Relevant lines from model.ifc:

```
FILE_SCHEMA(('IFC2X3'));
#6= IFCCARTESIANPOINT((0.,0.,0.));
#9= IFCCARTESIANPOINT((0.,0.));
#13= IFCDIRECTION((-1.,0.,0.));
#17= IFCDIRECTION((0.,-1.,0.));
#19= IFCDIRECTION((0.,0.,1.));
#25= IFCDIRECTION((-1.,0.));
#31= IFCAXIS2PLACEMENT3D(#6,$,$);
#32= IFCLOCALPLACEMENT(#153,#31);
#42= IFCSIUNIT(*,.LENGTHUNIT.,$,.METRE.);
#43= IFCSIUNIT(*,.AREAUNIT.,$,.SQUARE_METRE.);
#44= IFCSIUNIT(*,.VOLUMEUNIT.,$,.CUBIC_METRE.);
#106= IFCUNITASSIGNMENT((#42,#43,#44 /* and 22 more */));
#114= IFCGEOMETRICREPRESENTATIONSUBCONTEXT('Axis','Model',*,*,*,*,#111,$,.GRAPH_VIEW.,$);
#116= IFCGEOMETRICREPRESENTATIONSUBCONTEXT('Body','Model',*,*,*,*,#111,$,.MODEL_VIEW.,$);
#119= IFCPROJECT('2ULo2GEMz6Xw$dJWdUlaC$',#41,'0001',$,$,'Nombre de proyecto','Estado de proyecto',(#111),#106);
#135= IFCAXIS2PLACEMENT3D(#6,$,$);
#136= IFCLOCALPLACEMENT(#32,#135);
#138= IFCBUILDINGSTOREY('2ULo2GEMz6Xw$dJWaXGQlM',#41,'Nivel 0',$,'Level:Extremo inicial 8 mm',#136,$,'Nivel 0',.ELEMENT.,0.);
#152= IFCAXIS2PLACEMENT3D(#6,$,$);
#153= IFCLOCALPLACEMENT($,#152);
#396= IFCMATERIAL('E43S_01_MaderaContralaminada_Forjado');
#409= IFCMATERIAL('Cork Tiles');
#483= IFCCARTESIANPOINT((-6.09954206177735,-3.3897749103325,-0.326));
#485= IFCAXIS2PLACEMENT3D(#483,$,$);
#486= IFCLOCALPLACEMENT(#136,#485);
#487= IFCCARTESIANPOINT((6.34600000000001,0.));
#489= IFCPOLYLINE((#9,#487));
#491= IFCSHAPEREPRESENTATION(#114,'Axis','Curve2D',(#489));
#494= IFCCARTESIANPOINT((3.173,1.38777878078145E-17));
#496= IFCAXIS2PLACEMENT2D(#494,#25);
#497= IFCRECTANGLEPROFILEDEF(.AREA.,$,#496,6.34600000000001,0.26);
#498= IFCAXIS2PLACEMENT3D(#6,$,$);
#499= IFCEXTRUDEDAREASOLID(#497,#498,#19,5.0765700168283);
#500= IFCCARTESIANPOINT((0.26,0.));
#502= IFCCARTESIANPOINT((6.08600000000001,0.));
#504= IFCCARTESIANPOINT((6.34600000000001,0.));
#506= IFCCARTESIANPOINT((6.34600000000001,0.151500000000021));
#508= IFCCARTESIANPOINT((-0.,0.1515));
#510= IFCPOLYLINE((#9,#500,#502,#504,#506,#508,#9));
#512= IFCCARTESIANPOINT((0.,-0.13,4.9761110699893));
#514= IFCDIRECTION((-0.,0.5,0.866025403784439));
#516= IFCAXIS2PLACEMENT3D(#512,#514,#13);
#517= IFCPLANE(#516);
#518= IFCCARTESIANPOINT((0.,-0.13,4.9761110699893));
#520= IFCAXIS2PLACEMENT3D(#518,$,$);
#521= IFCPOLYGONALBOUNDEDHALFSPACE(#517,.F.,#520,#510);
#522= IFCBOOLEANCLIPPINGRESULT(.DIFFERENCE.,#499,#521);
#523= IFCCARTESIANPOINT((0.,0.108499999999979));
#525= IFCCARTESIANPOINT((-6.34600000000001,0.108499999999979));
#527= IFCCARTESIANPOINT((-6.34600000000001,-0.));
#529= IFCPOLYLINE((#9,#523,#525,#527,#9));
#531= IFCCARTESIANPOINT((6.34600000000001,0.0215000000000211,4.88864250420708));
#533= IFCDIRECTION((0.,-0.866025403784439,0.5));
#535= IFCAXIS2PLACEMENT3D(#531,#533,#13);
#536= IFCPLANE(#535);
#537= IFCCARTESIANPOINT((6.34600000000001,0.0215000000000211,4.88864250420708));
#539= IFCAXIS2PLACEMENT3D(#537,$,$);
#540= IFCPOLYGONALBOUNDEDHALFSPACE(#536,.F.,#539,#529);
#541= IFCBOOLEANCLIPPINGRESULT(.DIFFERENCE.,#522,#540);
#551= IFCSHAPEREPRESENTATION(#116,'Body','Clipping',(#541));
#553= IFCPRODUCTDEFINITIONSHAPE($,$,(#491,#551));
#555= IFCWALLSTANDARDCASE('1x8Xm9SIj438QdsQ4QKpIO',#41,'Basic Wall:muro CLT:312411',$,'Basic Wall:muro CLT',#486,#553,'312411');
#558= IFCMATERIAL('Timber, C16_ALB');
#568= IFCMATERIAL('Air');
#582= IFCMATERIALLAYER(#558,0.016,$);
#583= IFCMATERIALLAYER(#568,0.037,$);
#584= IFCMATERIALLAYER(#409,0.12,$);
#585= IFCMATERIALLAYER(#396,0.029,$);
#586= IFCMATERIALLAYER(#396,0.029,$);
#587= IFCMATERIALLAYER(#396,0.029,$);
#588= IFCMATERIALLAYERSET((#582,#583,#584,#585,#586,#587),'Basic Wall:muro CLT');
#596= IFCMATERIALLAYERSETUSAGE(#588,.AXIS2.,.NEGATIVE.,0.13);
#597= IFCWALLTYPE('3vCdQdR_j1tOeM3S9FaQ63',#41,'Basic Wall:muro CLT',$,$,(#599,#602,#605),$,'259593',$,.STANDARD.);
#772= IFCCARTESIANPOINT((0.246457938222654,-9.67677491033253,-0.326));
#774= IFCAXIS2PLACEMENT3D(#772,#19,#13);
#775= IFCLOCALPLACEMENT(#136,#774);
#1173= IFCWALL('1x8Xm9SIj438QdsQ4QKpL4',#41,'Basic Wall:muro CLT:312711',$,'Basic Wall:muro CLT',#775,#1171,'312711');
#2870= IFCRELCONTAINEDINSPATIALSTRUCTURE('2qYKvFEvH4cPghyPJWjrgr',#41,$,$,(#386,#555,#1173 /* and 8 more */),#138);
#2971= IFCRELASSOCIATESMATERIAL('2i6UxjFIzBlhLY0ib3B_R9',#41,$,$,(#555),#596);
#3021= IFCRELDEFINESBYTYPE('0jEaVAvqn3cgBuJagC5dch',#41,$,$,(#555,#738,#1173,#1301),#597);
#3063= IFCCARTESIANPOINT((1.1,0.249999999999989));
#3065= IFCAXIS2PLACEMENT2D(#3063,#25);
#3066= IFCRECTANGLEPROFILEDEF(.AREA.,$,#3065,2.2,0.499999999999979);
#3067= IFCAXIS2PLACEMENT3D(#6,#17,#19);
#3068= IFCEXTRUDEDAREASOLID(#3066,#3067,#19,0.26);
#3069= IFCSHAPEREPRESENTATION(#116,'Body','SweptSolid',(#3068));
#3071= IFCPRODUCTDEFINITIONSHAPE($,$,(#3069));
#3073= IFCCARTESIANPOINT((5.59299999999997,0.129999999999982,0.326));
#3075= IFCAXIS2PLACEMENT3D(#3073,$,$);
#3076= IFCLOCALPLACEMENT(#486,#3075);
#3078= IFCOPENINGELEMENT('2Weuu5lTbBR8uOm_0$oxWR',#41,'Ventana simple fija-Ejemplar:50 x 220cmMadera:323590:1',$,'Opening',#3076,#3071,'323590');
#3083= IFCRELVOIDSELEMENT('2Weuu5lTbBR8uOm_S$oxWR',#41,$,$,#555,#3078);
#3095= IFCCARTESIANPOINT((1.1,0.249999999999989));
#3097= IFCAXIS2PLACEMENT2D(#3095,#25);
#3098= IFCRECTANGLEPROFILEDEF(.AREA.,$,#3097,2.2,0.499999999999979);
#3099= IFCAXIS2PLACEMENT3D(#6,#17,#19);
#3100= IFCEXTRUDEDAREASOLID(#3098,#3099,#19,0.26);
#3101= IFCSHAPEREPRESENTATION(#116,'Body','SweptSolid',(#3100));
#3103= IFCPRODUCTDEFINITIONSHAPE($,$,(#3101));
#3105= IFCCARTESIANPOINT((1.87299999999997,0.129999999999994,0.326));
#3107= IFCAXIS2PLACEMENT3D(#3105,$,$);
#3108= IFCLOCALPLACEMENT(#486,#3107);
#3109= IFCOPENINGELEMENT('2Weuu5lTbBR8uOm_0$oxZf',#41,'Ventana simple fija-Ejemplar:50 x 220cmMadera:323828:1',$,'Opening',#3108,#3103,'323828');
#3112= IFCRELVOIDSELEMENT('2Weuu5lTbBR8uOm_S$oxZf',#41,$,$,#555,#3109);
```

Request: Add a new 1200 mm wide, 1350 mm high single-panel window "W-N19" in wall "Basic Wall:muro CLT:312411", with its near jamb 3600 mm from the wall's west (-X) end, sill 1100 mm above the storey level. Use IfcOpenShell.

```python
import numpy as np
import ifcopenshell
import ifcopenshell.api.feature
import ifcopenshell.api.geometry
import ifcopenshell.api.root
import ifcopenshell.api.spatial
import ifcopenshell.api.type
import ifcopenshell.geom
import ifcopenshell.util.element
import ifcopenshell.util.placement
import ifcopenshell.util.representation
import ifcopenshell.util.shape
import ifcopenshell.util.unit

model = ifcopenshell.open("model.ifc")
unit_scale = ifcopenshell.util.unit.calculate_unit_scale(model)
settings = ifcopenshell.geom.settings()


def volume(element):
    """Net volume in cubic metres, openings subtracted."""
    shape = ifcopenshell.geom.create_shape(settings, element)
    return ifcopenshell.util.shape.get_volume(shape.geometry)


wall = model.by_guid("1x8Xm9SIj438QdsQ4QKpIO")
storey = ifcopenshell.util.element.get_container(wall, ifc_class="IfcBuildingStorey")
context = ifcopenshell.util.representation.get_context(model, "Model", "Body", "MODEL_VIEW")
before = volume(wall)

width, height, from_end, sill = 1.2, 1.35, 3.6, 1.1  # metres

# The wall runs along its own X axis, and the end named is its -X end.
wall_shape = ifcopenshell.geom.create_shape(settings, wall)
x, y, z = ifcopenshell.util.shape.get_vertices(wall_shape.geometry).T
start = x.min() + from_end
face, thickness = float(y.min()), float(y.max() - y.min())
wall_matrix = ifcopenshell.util.placement.get_local_placement(wall.ObjectPlacement)
level = ifcopenshell.util.placement.get_local_placement(storey.ObjectPlacement)[2, 3]


def in_wall(x, y):
    """Placement at x, y metres in the wall's axes, at sill height."""
    matrix = wall_matrix.copy()
    matrix[:, 3] = wall_matrix @ np.array([x / unit_scale, y / unit_scale, 0.0, 1.0])
    matrix[2, 3] = level + sill / unit_scale
    return matrix


# Opening: a box that overshoots both wall faces by 50 mm.
opening = ifcopenshell.api.root.create_entity(model, ifc_class="IfcOpeningElement")
box = ifcopenshell.api.geometry.add_wall_representation(
    model, context=context, length=width, height=height, thickness=thickness + 0.1
)
ifcopenshell.api.geometry.assign_representation(model, product=opening, representation=box)
ifcopenshell.api.geometry.edit_object_placement(model, product=opening, matrix=in_wall(start, face - 0.05), is_si=False)
ifcopenshell.api.feature.add_feature(model, feature=opening, element=wall)

window = ifcopenshell.api.root.create_entity(model, ifc_class="IfcWindow", name="W-N19")
window.OverallWidth, window.OverallHeight = width / unit_scale, height / unit_scale
body = ifcopenshell.api.geometry.add_window_representation(
    model,
    context=context,
    overall_width=window.OverallWidth,
    overall_height=window.OverallHeight,
    partition_type="SINGLE_PANEL",
)
ifcopenshell.api.geometry.assign_representation(model, product=window, representation=body)
ifcopenshell.api.spatial.assign_container(model, products=[window], relating_structure=storey)
fills = ifcopenshell.api.feature.add_filling(model, opening=opening, element=window)
fills.OwnerHistory = window.OwnerHistory  # required in IFC2X3

# IFC2X3 keeps the operation on the window style.
style = ifcopenshell.api.root.create_entity(model, ifc_class="IfcWindowStyle", name="W-N19")
style.OperationType, style.ConstructionType = "SINGLE_PANEL", "NOTDEFINED"
style.ParameterTakesPrecedence = style.Sizeable = False
ifcopenshell.api.type.assign_type(model, related_objects=[window], relating_type=style)

# Centre the window in the wall's thickness.
ifcopenshell.api.geometry.edit_object_placement(model, product=window, matrix=in_wall(start, face), is_si=False)
window_shape = ifcopenshell.geom.create_shape(settings, window)
depth = ifcopenshell.util.shape.get_vertices(window_shape.geometry)[:, 1]
offset = face + thickness / 2 - (depth.min() + depth.max()) / 2
ifcopenshell.api.geometry.edit_object_placement(model, product=window, matrix=in_wall(start, offset), is_si=False)

after = volume(wall)

print(f"wall volume {before:.3f} -> {after:.3f} m3")

model.write("model_edited.ifc")
```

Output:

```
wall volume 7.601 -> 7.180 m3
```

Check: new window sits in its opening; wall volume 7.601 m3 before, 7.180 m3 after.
